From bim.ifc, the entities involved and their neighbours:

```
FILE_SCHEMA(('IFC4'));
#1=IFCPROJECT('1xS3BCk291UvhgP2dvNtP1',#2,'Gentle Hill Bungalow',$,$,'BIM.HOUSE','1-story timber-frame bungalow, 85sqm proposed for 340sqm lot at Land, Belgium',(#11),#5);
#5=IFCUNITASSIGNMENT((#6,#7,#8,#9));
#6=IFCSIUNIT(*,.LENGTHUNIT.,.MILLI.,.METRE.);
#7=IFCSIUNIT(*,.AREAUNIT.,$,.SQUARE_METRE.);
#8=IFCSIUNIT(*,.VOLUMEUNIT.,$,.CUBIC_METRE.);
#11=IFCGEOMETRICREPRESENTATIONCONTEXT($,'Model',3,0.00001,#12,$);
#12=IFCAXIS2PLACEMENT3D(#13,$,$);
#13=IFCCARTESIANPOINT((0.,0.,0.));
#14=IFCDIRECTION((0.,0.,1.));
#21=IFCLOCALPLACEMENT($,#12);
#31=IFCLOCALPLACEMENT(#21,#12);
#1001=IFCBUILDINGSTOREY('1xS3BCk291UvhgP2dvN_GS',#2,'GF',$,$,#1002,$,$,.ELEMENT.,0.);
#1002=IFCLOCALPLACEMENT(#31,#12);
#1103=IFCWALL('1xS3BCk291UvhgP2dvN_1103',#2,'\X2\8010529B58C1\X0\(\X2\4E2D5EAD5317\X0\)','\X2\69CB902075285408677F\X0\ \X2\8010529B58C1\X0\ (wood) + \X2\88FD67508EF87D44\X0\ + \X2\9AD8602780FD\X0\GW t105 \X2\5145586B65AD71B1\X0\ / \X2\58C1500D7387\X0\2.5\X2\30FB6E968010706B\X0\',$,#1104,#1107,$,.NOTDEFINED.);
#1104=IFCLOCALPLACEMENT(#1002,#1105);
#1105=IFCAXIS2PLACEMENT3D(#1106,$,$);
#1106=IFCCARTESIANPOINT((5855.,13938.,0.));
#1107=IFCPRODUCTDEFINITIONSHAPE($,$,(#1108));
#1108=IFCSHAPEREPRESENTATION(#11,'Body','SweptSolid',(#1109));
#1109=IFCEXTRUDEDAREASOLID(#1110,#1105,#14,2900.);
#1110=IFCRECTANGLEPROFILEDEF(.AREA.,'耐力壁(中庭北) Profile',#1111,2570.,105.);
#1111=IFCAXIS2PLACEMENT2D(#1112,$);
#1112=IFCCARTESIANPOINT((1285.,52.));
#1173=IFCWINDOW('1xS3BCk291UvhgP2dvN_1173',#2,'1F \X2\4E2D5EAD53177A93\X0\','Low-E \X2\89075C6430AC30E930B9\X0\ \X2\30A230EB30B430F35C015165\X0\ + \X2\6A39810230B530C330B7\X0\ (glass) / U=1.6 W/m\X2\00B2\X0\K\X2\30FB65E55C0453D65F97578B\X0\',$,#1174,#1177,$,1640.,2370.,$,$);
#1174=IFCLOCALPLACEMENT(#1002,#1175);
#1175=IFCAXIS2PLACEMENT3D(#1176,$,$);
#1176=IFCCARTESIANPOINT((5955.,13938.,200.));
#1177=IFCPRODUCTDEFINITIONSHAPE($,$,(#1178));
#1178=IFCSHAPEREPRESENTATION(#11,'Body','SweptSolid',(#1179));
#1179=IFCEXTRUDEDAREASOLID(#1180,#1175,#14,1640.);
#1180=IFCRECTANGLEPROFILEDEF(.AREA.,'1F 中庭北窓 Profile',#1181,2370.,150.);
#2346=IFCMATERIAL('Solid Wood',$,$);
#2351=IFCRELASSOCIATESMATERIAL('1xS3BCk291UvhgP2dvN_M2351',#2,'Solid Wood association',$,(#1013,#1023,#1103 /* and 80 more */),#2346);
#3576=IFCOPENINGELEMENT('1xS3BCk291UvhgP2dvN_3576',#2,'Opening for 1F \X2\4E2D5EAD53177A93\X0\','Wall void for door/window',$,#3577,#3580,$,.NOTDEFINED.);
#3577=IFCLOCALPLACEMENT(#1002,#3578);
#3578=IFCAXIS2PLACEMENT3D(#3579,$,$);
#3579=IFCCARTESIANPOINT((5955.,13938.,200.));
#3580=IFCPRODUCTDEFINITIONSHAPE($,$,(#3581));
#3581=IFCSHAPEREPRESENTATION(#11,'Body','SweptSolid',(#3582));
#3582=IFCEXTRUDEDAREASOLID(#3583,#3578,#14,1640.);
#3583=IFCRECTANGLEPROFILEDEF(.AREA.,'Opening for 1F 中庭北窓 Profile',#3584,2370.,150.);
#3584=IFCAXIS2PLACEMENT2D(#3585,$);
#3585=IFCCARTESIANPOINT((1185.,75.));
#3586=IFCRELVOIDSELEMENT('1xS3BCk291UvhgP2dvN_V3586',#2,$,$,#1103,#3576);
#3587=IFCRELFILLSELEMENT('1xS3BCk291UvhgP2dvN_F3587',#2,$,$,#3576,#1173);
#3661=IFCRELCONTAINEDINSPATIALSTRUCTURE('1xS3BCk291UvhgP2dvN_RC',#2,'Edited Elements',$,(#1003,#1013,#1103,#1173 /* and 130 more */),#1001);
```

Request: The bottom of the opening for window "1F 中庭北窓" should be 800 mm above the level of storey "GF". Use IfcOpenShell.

```python
import numpy as np
import ifcopenshell
import ifcopenshell.api.geometry
import ifcopenshell.geom
import ifcopenshell.util.element
import ifcopenshell.util.placement
import ifcopenshell.util.shape
import ifcopenshell.util.unit

model = ifcopenshell.open("bim.ifc")
unit_scale = ifcopenshell.util.unit.calculate_unit_scale(model)

window = model.by_guid("1xS3BCk291UvhgP2dvN_1173")
opening = window.FillsVoids[0].RelatingOpeningElement
storey = ifcopenshell.util.element.get_container(window, ifc_class="IfcBuildingStorey")
level = ifcopenshell.util.placement.get_local_placement(storey.ObjectPlacement)[2, 3]

# The opening's origin need not be at the sill, so measure its lowest point.
shape = ifcopenshell.geom.create_shape(ifcopenshell.geom.settings(), opening)
bottom = ifcopenshell.util.shape.get_shape_bottom_elevation(shape, shape.geometry) / unit_scale
dz = level + 800.0 - bottom

shift = np.array([0.0, 0.0, dz])
# The window is not placed relative to its opening, so move both.
for product in (opening, window):
    matrix = ifcopenshell.util.placement.get_local_placement(product.ObjectPlacement)
    matrix[:3, 3] += shift
    ifcopenshell.api.geometry.edit_object_placement(model, product=product, matrix=matrix, is_si=False)

print(f"moved by {dz * unit_scale:+.3f} m")

model.write("bim_rev.ifc")
```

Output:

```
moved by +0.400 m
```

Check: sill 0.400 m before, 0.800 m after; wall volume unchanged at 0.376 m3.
